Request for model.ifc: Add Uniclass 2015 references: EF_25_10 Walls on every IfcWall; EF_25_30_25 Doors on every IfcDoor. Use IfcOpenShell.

First a look at what the model holds.

```python
import ifcopenshell

model = ifcopenshell.open("model.ifc")
print(model.schema)
print("classifications:", [c.Name for c in model.by_type("IfcClassification")])
for ifc_class in ("IfcDoor", "IfcRoof", "IfcStair", "IfcWall", "IfcWindow"):
    print(ifc_class, len(model.by_type(ifc_class)))
```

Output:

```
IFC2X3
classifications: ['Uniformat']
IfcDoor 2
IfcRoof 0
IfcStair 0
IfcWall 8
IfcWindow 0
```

```python
import ifcopenshell
import ifcopenshell.api.classification

model = ifcopenshell.open("model.ifc")

# IFC2X3 requires Source and Edition and has no link from the project to the system.
system = model.create_entity("IfcClassification", Source="NBS", Edition="2015", Name="Uniclass 2015")

codes = {
    "IfcWall": ("EF_25_10", "Walls"),
    "IfcDoor": ("EF_25_30_25", "Doors"),
}
for ifc_class, (code, name) in codes.items():
    products = model.by_type(ifc_class)
    ifcopenshell.api.classification.add_reference(
        model, products=products, classification=system, identification=code, name=name
    )
    print(code, len(products))

model.write("model_v2.ifc")
```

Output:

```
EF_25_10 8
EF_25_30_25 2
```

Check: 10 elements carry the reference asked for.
